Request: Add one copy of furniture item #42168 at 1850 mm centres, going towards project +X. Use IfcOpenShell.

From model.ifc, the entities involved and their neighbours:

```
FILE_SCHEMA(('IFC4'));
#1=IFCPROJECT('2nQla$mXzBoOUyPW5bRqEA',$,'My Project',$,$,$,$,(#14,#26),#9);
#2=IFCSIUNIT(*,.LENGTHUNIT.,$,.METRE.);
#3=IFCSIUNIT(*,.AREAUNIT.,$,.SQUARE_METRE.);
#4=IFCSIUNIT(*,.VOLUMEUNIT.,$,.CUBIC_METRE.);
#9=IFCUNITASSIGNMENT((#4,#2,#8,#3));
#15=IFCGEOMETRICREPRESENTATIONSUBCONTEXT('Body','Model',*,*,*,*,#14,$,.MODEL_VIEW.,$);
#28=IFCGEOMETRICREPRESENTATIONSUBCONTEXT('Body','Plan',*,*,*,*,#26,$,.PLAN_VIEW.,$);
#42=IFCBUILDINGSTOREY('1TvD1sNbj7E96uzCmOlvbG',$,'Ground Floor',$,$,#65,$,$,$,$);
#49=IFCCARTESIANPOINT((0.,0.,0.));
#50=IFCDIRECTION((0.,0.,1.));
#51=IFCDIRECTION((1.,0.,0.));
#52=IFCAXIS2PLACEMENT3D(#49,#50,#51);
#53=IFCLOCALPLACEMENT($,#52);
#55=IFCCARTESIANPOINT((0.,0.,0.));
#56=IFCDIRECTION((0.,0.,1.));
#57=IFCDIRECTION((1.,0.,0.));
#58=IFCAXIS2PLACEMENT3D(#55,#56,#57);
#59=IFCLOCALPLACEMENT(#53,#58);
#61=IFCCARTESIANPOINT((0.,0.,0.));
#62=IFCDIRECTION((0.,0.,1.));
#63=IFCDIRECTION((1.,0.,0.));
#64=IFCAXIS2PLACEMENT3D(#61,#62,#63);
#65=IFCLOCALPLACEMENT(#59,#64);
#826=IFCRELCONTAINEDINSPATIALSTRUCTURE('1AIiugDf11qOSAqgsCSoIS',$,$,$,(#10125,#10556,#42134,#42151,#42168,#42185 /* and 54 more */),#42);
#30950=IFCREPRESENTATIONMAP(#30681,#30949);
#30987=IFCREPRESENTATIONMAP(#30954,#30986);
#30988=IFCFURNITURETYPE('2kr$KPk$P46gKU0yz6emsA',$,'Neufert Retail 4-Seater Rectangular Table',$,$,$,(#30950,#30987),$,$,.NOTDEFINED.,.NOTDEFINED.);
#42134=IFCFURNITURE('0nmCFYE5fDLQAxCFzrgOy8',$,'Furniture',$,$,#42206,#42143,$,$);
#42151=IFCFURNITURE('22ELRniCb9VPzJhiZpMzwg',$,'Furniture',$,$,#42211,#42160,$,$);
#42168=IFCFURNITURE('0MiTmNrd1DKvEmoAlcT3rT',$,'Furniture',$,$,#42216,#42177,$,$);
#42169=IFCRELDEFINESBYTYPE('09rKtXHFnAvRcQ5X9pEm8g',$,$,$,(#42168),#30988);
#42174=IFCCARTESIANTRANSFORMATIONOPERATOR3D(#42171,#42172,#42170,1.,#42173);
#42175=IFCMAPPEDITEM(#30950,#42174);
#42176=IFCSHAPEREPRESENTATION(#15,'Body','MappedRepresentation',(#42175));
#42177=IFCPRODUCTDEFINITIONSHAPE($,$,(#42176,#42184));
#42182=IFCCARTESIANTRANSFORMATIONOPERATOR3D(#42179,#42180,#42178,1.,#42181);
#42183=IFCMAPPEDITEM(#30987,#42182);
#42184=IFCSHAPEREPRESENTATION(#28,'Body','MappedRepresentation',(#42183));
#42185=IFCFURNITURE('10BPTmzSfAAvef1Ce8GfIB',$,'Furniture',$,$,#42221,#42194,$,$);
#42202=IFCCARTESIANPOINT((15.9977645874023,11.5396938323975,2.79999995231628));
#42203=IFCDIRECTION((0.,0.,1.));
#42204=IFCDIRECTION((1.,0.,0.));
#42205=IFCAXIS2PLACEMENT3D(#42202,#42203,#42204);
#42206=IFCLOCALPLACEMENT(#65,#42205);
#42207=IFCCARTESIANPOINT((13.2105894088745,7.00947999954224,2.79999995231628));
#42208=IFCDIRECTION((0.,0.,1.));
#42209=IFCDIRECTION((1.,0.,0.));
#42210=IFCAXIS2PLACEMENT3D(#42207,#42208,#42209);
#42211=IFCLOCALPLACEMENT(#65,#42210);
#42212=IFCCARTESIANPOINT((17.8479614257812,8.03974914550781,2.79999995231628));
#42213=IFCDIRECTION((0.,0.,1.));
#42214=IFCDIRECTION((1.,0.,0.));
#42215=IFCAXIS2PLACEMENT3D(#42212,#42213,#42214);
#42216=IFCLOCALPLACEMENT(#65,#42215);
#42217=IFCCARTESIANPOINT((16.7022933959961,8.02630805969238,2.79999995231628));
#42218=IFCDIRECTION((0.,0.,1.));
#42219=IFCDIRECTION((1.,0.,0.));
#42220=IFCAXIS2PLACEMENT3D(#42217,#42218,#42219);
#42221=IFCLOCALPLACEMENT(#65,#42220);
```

```python
import numpy as np
import ifcopenshell
import ifcopenshell.api.geometry
import ifcopenshell.api.root
import ifcopenshell.util.element
import ifcopenshell.util.placement
import ifcopenshell.util.unit

model = ifcopenshell.open("model.ifc")
unit_scale = ifcopenshell.util.unit.calculate_unit_scale(model)

source = model.by_guid("0MiTmNrd1DKvEmoAlcT3rT")
base = ifcopenshell.util.placement.get_local_placement(source.ObjectPlacement)
step = np.array([1.0, 0.0, 0.0]) * 1.85 / unit_scale

for i in range(1, 2):
    copy = ifcopenshell.api.root.copy_class(model, product=source)
    copy.Representation = ifcopenshell.util.element.copy_deep(
        model, source.Representation, exclude=["IfcGeometricRepresentationContext", "IfcRepresentationMap"]
    )
    matrix = base.copy()
    matrix[:3, 3] += i * step
    print("added at", matrix[:3, 3].round(3) + 0.0)
    ifcopenshell.api.geometry.edit_object_placement(model, product=copy, matrix=matrix, is_si=False)

model.write("model-out.ifc")
```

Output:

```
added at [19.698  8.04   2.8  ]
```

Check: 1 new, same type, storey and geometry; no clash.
